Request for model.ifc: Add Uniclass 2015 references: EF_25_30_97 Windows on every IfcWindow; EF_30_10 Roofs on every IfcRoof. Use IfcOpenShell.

First a look at what the model holds.

```python
import ifcopenshell

model = ifcopenshell.open("model.ifc")
print(model.schema)
print("classifications:", [c.Name for c in model.by_type("IfcClassification")])
for ifc_class in ("IfcDoor", "IfcRoof", "IfcStair", "IfcWall", "IfcWindow"):
    print(ifc_class, len(model.by_type(ifc_class)))
```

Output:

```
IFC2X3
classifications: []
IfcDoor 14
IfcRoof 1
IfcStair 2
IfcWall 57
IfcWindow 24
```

```python
import ifcopenshell
import ifcopenshell.api.classification

model = ifcopenshell.open("model.ifc")

# IFC2X3 requires Source and Edition and has no link from the project to the system.
system = model.create_entity("IfcClassification", Source="NBS", Edition="2015", Name="Uniclass 2015")

codes = {
    "IfcWindow": ("EF_25_30_97", "Windows"),
    "IfcRoof": ("EF_30_10", "Roofs"),
}
for ifc_class, (code, name) in codes.items():
    products = model.by_type(ifc_class)
    ifcopenshell.api.classification.add_reference(
        model, products=products, classification=system, identification=code, name=name
    )
    print(code, len(products))

model.write("model_rev.ifc")
```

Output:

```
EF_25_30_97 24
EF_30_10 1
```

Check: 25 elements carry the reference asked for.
